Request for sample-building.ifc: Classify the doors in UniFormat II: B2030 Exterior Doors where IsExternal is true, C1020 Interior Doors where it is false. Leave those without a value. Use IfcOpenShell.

First a look at what the model holds.

```python
import ifcopenshell
import ifcopenshell.util.element

model = ifcopenshell.open("sample-building.ifc")
print(model.schema)
print("classifications:", [c.Name for c in model.by_type("IfcClassification")])
values = [ifcopenshell.util.element.get_pset(e, "Pset_DoorCommon", "IsExternal") for e in model.by_type("IfcDoor")]
for value in (True, False, None):
    print("IsExternal", value, values.count(value))
```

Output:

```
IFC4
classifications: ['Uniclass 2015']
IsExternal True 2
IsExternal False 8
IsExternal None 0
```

```python
import ifcopenshell
import ifcopenshell.api.classification
import ifcopenshell.util.element

model = ifcopenshell.open("sample-building.ifc")

system = ifcopenshell.api.classification.add_classification(model, classification="UniFormat II")

doors = model.by_type("IfcDoor")
external = {e: ifcopenshell.util.element.get_pset(e, "Pset_DoorCommon", "IsExternal") for e in doors}
for flag, code, name in ((True, "B2030", "Exterior Doors"), (False, "C1020", "Interior Doors")):
    products = [e for e in doors if external[e] is flag]
    ifcopenshell.api.classification.add_reference(
        model, products=products, classification=system, identification=code, name=name
    )
    print(code, len(products))

model.write("sample-building_updated.ifc")
```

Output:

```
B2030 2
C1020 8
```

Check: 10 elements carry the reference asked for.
